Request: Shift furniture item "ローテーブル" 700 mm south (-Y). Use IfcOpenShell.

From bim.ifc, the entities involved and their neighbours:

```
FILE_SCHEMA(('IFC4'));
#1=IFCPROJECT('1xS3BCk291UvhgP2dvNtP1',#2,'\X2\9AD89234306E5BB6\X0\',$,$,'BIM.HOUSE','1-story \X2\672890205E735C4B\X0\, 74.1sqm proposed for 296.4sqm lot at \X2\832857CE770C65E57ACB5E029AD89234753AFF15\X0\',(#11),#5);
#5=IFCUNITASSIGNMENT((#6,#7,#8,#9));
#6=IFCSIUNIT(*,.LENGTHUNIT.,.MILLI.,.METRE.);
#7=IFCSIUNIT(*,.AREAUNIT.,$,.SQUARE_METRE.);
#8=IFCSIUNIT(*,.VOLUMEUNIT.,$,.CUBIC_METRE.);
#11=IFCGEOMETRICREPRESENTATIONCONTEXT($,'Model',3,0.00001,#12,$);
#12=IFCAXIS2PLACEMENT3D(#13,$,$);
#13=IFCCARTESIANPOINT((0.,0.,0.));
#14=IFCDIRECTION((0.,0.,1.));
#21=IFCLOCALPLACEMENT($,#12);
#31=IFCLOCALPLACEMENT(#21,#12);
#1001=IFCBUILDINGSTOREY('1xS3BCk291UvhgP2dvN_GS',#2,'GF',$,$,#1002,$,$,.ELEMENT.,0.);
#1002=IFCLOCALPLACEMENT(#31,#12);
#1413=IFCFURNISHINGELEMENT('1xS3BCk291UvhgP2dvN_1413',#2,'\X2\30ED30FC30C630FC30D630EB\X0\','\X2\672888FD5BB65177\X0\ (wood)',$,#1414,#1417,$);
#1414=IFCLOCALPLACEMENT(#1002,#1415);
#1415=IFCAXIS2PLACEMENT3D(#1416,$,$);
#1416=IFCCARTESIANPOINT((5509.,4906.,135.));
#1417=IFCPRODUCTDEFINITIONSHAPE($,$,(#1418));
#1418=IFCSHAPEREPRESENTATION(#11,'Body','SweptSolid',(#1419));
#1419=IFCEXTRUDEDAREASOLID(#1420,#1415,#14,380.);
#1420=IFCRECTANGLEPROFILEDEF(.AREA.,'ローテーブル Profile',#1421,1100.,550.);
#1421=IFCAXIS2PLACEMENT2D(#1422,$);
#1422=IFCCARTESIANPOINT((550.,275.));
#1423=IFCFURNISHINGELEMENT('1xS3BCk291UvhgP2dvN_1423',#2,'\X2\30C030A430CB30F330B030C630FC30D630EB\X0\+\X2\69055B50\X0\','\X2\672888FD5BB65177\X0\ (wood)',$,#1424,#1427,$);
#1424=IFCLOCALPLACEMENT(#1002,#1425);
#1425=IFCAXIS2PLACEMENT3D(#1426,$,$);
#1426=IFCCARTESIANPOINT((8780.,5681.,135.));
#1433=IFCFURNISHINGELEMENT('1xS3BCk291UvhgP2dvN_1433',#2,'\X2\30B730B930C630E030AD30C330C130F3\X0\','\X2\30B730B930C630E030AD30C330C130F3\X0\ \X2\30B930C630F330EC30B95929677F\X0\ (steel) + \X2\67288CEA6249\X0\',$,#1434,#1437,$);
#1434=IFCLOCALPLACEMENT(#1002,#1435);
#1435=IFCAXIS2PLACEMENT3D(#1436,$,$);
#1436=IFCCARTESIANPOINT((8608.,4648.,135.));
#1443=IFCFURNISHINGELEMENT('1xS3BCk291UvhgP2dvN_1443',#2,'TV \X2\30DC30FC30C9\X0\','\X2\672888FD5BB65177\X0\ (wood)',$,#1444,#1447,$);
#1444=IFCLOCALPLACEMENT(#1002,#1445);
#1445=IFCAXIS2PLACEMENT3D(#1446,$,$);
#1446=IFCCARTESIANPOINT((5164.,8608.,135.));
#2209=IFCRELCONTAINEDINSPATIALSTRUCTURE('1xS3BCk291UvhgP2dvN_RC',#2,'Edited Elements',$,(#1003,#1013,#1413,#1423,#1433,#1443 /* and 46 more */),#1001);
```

```python
import ifcopenshell
import ifcopenshell.api.geometry
import ifcopenshell.util.placement
import ifcopenshell.util.unit

model = ifcopenshell.open("bim.ifc")
unit_scale = ifcopenshell.util.unit.calculate_unit_scale(model)

item = model.by_guid("1xS3BCk291UvhgP2dvN_1413")
matrix = ifcopenshell.util.placement.get_local_placement(item.ObjectPlacement)
matrix[1, 3] -= 0.7 / unit_scale
ifcopenshell.api.geometry.edit_object_placement(model, product=item, matrix=matrix, is_si=False)

print(ifcopenshell.util.placement.get_local_placement(item.ObjectPlacement).round(3) + 0.0)

model.write("bim_rev.ifc")
```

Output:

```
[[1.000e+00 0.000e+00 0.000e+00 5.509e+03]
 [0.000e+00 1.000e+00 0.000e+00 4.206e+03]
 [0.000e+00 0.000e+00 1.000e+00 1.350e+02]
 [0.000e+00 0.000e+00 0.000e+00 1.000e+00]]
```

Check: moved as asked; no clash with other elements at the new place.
